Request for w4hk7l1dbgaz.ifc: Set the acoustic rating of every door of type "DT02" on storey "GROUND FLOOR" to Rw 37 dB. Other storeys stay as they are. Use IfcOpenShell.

First a look at what the model holds.

```python
import ifcopenshell
import ifcopenshell.util.element

model = ifcopenshell.open("w4hk7l1dbgaz.ifc")
print(model.schema)
storey = next(s for s in model.by_type("IfcBuildingStorey") if s.Name == "GROUND FLOOR")
doors = [e for e in ifcopenshell.util.element.get_decomposition(storey) if e.is_a("IfcDoor")]
seen = {}
for e in doors:
    element_type = ifcopenshell.util.element.get_type(e)
    key = (element_type.Name if element_type != e and element_type else None, ifcopenshell.util.element.get_pset(e, "Pset_DoorCommon", "AcousticRating"))
    seen[key] = seen.get(key, 0) + 1
for (name, value), count in sorted(seen.items(), key=str):
    print(count, "x", name, "|", value)
```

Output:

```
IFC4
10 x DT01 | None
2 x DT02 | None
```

```python
import ifcopenshell
import ifcopenshell.api.pset
import ifcopenshell.util.element

model = ifcopenshell.open("w4hk7l1dbgaz.ifc")

storey = next(s for s in model.by_type("IfcBuildingStorey") if s.Name == "GROUND FLOOR")
doors = [e for e in ifcopenshell.util.element.get_decomposition(storey) if e.is_a("IfcDoor")]

count = 0
for e in doors:
    element_type = ifcopenshell.util.element.get_type(e)
    if element_type in (None, e) or element_type.Name != "DT02":
        continue
    # add_pset returns the element's existing set when there is one.
    pset = ifcopenshell.api.pset.add_pset(model, product=e, name="Pset_DoorCommon")
    ifcopenshell.api.pset.edit_pset(model, pset=pset, properties={"AcousticRating": "Rw 37 dB"})
    count += 1

print(count, "doors updated")

model.write("w4hk7l1dbgaz_v2.ifc")
```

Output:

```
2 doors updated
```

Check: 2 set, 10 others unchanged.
